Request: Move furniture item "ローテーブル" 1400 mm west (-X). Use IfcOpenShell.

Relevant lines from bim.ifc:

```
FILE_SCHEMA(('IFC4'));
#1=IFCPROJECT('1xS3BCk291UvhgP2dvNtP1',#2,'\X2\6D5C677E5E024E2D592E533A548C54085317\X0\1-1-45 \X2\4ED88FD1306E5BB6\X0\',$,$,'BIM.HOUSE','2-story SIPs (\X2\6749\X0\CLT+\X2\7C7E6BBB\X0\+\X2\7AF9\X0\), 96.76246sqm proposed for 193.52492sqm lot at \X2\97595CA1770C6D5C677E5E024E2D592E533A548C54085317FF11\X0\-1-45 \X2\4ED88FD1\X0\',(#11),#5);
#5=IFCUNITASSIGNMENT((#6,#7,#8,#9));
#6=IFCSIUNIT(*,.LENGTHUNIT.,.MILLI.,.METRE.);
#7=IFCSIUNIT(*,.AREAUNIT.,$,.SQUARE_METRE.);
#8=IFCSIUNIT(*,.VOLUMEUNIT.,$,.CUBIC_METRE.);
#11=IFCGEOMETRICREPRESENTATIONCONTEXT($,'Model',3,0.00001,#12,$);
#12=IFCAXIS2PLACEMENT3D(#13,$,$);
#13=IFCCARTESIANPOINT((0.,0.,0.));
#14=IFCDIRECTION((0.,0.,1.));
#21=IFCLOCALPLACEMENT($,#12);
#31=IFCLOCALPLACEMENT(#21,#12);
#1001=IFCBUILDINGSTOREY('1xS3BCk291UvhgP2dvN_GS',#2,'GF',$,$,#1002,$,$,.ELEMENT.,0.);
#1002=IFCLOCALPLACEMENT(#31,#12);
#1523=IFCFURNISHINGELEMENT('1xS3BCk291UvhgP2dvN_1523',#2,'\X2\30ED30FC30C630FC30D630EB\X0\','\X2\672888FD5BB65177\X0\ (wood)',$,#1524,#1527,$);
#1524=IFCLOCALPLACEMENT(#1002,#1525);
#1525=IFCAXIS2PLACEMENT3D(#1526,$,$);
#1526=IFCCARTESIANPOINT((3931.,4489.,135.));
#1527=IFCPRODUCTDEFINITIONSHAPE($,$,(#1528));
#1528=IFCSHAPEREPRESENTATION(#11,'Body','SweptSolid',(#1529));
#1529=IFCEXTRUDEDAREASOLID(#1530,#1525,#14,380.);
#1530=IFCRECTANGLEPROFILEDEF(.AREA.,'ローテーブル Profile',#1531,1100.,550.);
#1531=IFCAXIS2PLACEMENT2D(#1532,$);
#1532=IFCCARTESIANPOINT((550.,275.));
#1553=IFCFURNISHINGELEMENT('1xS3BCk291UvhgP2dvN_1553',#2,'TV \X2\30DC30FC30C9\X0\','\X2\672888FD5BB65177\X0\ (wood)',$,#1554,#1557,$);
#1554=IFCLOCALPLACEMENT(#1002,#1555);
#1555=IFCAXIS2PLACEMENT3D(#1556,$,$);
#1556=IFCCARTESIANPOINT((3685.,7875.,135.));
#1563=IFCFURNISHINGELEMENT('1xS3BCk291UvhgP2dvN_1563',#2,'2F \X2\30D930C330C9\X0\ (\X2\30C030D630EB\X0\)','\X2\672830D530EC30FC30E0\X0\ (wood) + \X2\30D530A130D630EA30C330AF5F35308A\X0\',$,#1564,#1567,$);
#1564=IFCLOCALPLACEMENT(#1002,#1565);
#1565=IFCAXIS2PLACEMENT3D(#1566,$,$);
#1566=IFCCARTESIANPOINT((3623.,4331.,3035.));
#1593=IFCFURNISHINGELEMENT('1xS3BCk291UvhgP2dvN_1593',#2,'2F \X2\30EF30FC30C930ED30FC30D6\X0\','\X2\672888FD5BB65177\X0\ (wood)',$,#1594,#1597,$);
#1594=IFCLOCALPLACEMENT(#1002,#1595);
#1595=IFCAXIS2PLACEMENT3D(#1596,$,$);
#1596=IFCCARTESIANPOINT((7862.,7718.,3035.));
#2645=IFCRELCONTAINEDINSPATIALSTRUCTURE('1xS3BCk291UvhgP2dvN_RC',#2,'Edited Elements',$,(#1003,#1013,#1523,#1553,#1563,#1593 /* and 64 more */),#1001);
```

```python
import ifcopenshell
import ifcopenshell.api.geometry
import ifcopenshell.util.placement

model = ifcopenshell.open("bim.ifc")

item = model.by_guid("1xS3BCk291UvhgP2dvN_1523")
matrix = ifcopenshell.util.placement.get_local_placement(item.ObjectPlacement)
matrix[0, 3] -= 1400.0
ifcopenshell.api.geometry.edit_object_placement(model, product=item, matrix=matrix, is_si=False)

print(ifcopenshell.util.placement.get_local_placement(item.ObjectPlacement).round(3) + 0.0)

model.write("bim-out.ifc")
```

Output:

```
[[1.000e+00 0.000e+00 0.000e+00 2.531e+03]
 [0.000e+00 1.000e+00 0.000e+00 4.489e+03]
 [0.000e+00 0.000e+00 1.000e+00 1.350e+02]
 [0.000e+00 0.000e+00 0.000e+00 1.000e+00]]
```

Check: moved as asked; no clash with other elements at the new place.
